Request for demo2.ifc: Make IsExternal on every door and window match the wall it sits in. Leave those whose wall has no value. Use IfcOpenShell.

First a look at what the model holds.

```python
import ifcopenshell
import ifcopenshell.util.element

model = ifcopenshell.open("demo2.ifc")
print(model.schema)
seen = {}
for e in model.by_type("IfcDoor") + model.by_type("IfcWindow"):
    if not e.FillsVoids:
        continue
    host = e.FillsVoids[0].RelatingOpeningElement.VoidsElements[0].RelatingBuildingElement
    own = ifcopenshell.util.element.get_pset(e, f"Pset_{e.is_a()[3:].removesuffix('StandardCase')}Common", "IsExternal")
    wall = ifcopenshell.util.element.get_pset(host, "Pset_WallCommon", "IsExternal")
    seen[e.is_a(), own, wall] = seen.get((e.is_a(), own, wall), 0) + 1
for (cls, own, wall), count in sorted(seen.items(), key=str):
    print(count, cls, "IsExternal:", own, "| host wall:", wall)
```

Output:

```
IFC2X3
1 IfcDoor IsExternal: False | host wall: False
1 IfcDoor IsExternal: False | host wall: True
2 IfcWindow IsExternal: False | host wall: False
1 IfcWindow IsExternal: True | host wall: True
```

```python
import ifcopenshell
import ifcopenshell.api.pset
import ifcopenshell.util.element

model = ifcopenshell.open("demo2.ifc")

count = 0
for ifc_class, pset_name in (("IfcDoor", "Pset_DoorCommon"), ("IfcWindow", "Pset_WindowCommon")):
    for e in model.by_type(ifc_class):
        if not e.FillsVoids:
            continue
        host = e.FillsVoids[0].RelatingOpeningElement.VoidsElements[0].RelatingBuildingElement
        external = ifcopenshell.util.element.get_pset(host, "Pset_WallCommon", "IsExternal")
        if external is None or ifcopenshell.util.element.get_pset(e, pset_name, "IsExternal") == external:
            continue
        pset = ifcopenshell.api.pset.add_pset(model, product=e, name=pset_name)
        ifcopenshell.api.pset.edit_pset(model, pset=pset, properties={"IsExternal": external})
        count += 1

print(count, "updated")

model.write("demo2_updated.ifc")
```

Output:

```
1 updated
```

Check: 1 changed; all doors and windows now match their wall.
